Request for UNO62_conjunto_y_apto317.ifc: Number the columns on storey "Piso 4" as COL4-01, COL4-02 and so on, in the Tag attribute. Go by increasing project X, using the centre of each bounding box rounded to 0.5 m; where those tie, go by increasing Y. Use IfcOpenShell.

First a look at what the model holds.

```python
import ifcopenshell
import ifcopenshell.util.element
import ifcopenshell.util.placement

model = ifcopenshell.open("UNO62_conjunto_y_apto317.ifc")
print(model.schema)
storey = next(s for s in model.by_type("IfcBuildingStorey") if s.Name == "Piso 4")
columns = [e for e in ifcopenshell.util.element.get_decomposition(storey) if e.is_a("IfcColumn")]
for e in sorted(columns, key=lambda e: e.id()):
    origin = ifcopenshell.util.placement.get_local_placement(e.ObjectPlacement)[:3, 3]
    print(e.id(), e.Tag, e.Name, origin.round(2) + 0.0, sep=" | ")
```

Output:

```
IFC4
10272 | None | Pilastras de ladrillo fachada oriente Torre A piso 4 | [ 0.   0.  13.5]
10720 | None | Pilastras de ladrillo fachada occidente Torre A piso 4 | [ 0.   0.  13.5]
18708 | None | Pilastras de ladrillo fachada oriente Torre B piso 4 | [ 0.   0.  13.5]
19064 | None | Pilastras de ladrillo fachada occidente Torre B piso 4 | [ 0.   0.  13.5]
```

```python
import ifcopenshell
import ifcopenshell.geom
import ifcopenshell.util.element
import ifcopenshell.util.shape

model = ifcopenshell.open("UNO62_conjunto_y_apto317.ifc")
settings = ifcopenshell.geom.settings()
settings.set("use-world-coords", True)


def centre(element):
    shape = ifcopenshell.geom.create_shape(settings, element)
    return ifcopenshell.util.shape.get_bbox_centroid(shape.geometry)


storey = next(s for s in model.by_type("IfcBuildingStorey") if s.Name == "Piso 4")
columns = [e for e in ifcopenshell.util.element.get_decomposition(storey) if e.is_a("IfcColumn")]

# Insertion points can sit at a corner or the storey origin, so sort by the geometry (in metres).
centres = {e: centre(e) for e in columns}
columns.sort(key=lambda e: (round(centres[e][0] / 0.5), centres[e][1]))

for i, e in enumerate(columns, start=1):
    number = f"COL4-{i:02d}"
    e.Tag = number
    print(e.id(), number)

model.write("UNO62_conjunto_y_apto317_edited.ifc")
```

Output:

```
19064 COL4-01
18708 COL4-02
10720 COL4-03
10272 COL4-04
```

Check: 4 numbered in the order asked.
